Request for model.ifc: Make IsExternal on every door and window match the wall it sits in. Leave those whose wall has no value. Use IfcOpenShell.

First a look at what the model holds.

```python
import ifcopenshell
import ifcopenshell.util.element

model = ifcopenshell.open("model.ifc")
print(model.schema)
seen = {}
for e in model.by_type("IfcDoor") + model.by_type("IfcWindow"):
    if not e.FillsVoids:
        continue
    host = e.FillsVoids[0].RelatingOpeningElement.VoidsElements[0].RelatingBuildingElement
    own = ifcopenshell.util.element.get_pset(e, f"Pset_{e.is_a()[3:].removesuffix('StandardCase')}Common", "IsExternal")
    wall = ifcopenshell.util.element.get_pset(host, "Pset_WallCommon", "IsExternal")
    seen[e.is_a(), own, wall] = seen.get((e.is_a(), own, wall), 0) + 1
for (cls, own, wall), count in sorted(seen.items(), key=str):
    print(count, cls, "IsExternal:", own, "| host wall:", wall)
```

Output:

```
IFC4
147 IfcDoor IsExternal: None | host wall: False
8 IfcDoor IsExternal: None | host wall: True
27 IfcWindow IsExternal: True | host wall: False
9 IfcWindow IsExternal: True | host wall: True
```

```python
import ifcopenshell
import ifcopenshell.api.pset
import ifcopenshell.util.element

model = ifcopenshell.open("model.ifc")

count = 0
for ifc_class, pset_name in (("IfcDoor", "Pset_DoorCommon"), ("IfcWindow", "Pset_WindowCommon")):
    for e in model.by_type(ifc_class):
        if not e.FillsVoids:
            continue
        host = e.FillsVoids[0].RelatingOpeningElement.VoidsElements[0].RelatingBuildingElement
        external = ifcopenshell.util.element.get_pset(host, "Pset_WallCommon", "IsExternal")
        if external is None or ifcopenshell.util.element.get_pset(e, pset_name, "IsExternal") == external:
            continue
        pset = ifcopenshell.api.pset.add_pset(model, product=e, name=pset_name)
        ifcopenshell.api.pset.edit_pset(model, pset=pset, properties={"IsExternal": external})
        count += 1

print(count, "updated")

model.write("model_rev.ifc")
```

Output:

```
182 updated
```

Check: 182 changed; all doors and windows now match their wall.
